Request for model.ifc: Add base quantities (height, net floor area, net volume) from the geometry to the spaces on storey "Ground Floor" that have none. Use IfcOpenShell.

First a look at what the model holds.

```python
import ifcopenshell
import ifcopenshell.util.element
import ifcopenshell.util.unit

model = ifcopenshell.open("model.ifc")
print(model.schema)
for unit_type in ("LENGTHUNIT", "AREAUNIT", "VOLUMEUNIT"):
    print(unit_type, ifcopenshell.util.unit.calculate_unit_scale(model, unit_type))
storey = next(s for s in model.by_type("IfcBuildingStorey") if s.Name == "Ground Floor")
spaces = [e for e in ifcopenshell.util.element.get_decomposition(storey) if e.is_a("IfcSpace")]
for e in sorted(spaces, key=lambda e: e.id()):
    print(e.id(), e.is_a(), e.Name, list(ifcopenshell.util.element.get_psets(e, qtos_only=True)), sep=" | ")
```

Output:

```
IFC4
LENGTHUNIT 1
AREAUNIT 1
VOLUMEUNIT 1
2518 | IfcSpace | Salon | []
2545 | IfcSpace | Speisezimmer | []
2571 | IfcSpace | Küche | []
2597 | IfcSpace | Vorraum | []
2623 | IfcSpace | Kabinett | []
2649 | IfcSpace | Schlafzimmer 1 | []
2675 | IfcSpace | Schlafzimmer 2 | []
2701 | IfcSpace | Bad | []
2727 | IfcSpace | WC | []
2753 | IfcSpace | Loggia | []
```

```python
import ifcopenshell
import ifcopenshell.api.pset
import ifcopenshell.geom
import ifcopenshell.util.element
import ifcopenshell.util.shape
import ifcopenshell.util.unit

model = ifcopenshell.open("model.ifc")
unit_scale = ifcopenshell.util.unit.calculate_unit_scale(model)
area_scale = ifcopenshell.util.unit.calculate_unit_scale(model, "AREAUNIT")
volume_scale = ifcopenshell.util.unit.calculate_unit_scale(model, "VOLUMEUNIT")
settings = ifcopenshell.geom.settings()

storey = next(s for s in model.by_type("IfcBuildingStorey") if s.Name == "Ground Floor")
spaces = [e for e in ifcopenshell.util.element.get_decomposition(storey) if e.is_a("IfcSpace")]

for e in sorted(spaces, key=lambda e: e.id()):
    if ifcopenshell.util.element.get_psets(e, qtos_only=True, should_inherit=False):
        continue
    # Geometry comes back in metres, in the element's own axes.
    shape = ifcopenshell.geom.create_shape(settings, e)
    values = {
        "Height": ifcopenshell.util.shape.get_z(shape.geometry) / unit_scale,
        "NetFloorArea": ifcopenshell.util.shape.get_footprint_area(shape.geometry) / area_scale,
        "NetVolume": ifcopenshell.util.shape.get_volume(shape.geometry) / volume_scale,
    }
    qto = ifcopenshell.api.pset.add_qto(model, product=e, name="Qto_SpaceBaseQuantities")
    ifcopenshell.api.pset.edit_qto(model, qto=qto, properties=values)
    print(e.id(), {k: round(v, 3) for k, v in values.items()})

model.write("model_v2.ifc")
```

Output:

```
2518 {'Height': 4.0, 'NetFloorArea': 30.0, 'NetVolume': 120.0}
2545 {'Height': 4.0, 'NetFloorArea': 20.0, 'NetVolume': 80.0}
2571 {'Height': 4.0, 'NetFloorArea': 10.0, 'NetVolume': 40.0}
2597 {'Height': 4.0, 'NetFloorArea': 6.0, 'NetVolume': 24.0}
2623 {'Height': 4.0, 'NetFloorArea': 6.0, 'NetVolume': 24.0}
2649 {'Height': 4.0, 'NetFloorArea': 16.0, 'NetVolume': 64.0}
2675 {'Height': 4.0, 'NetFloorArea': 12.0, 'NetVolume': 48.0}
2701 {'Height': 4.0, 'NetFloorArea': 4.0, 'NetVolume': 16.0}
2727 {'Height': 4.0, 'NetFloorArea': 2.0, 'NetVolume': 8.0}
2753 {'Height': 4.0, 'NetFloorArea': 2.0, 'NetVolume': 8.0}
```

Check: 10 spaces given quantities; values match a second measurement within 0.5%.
